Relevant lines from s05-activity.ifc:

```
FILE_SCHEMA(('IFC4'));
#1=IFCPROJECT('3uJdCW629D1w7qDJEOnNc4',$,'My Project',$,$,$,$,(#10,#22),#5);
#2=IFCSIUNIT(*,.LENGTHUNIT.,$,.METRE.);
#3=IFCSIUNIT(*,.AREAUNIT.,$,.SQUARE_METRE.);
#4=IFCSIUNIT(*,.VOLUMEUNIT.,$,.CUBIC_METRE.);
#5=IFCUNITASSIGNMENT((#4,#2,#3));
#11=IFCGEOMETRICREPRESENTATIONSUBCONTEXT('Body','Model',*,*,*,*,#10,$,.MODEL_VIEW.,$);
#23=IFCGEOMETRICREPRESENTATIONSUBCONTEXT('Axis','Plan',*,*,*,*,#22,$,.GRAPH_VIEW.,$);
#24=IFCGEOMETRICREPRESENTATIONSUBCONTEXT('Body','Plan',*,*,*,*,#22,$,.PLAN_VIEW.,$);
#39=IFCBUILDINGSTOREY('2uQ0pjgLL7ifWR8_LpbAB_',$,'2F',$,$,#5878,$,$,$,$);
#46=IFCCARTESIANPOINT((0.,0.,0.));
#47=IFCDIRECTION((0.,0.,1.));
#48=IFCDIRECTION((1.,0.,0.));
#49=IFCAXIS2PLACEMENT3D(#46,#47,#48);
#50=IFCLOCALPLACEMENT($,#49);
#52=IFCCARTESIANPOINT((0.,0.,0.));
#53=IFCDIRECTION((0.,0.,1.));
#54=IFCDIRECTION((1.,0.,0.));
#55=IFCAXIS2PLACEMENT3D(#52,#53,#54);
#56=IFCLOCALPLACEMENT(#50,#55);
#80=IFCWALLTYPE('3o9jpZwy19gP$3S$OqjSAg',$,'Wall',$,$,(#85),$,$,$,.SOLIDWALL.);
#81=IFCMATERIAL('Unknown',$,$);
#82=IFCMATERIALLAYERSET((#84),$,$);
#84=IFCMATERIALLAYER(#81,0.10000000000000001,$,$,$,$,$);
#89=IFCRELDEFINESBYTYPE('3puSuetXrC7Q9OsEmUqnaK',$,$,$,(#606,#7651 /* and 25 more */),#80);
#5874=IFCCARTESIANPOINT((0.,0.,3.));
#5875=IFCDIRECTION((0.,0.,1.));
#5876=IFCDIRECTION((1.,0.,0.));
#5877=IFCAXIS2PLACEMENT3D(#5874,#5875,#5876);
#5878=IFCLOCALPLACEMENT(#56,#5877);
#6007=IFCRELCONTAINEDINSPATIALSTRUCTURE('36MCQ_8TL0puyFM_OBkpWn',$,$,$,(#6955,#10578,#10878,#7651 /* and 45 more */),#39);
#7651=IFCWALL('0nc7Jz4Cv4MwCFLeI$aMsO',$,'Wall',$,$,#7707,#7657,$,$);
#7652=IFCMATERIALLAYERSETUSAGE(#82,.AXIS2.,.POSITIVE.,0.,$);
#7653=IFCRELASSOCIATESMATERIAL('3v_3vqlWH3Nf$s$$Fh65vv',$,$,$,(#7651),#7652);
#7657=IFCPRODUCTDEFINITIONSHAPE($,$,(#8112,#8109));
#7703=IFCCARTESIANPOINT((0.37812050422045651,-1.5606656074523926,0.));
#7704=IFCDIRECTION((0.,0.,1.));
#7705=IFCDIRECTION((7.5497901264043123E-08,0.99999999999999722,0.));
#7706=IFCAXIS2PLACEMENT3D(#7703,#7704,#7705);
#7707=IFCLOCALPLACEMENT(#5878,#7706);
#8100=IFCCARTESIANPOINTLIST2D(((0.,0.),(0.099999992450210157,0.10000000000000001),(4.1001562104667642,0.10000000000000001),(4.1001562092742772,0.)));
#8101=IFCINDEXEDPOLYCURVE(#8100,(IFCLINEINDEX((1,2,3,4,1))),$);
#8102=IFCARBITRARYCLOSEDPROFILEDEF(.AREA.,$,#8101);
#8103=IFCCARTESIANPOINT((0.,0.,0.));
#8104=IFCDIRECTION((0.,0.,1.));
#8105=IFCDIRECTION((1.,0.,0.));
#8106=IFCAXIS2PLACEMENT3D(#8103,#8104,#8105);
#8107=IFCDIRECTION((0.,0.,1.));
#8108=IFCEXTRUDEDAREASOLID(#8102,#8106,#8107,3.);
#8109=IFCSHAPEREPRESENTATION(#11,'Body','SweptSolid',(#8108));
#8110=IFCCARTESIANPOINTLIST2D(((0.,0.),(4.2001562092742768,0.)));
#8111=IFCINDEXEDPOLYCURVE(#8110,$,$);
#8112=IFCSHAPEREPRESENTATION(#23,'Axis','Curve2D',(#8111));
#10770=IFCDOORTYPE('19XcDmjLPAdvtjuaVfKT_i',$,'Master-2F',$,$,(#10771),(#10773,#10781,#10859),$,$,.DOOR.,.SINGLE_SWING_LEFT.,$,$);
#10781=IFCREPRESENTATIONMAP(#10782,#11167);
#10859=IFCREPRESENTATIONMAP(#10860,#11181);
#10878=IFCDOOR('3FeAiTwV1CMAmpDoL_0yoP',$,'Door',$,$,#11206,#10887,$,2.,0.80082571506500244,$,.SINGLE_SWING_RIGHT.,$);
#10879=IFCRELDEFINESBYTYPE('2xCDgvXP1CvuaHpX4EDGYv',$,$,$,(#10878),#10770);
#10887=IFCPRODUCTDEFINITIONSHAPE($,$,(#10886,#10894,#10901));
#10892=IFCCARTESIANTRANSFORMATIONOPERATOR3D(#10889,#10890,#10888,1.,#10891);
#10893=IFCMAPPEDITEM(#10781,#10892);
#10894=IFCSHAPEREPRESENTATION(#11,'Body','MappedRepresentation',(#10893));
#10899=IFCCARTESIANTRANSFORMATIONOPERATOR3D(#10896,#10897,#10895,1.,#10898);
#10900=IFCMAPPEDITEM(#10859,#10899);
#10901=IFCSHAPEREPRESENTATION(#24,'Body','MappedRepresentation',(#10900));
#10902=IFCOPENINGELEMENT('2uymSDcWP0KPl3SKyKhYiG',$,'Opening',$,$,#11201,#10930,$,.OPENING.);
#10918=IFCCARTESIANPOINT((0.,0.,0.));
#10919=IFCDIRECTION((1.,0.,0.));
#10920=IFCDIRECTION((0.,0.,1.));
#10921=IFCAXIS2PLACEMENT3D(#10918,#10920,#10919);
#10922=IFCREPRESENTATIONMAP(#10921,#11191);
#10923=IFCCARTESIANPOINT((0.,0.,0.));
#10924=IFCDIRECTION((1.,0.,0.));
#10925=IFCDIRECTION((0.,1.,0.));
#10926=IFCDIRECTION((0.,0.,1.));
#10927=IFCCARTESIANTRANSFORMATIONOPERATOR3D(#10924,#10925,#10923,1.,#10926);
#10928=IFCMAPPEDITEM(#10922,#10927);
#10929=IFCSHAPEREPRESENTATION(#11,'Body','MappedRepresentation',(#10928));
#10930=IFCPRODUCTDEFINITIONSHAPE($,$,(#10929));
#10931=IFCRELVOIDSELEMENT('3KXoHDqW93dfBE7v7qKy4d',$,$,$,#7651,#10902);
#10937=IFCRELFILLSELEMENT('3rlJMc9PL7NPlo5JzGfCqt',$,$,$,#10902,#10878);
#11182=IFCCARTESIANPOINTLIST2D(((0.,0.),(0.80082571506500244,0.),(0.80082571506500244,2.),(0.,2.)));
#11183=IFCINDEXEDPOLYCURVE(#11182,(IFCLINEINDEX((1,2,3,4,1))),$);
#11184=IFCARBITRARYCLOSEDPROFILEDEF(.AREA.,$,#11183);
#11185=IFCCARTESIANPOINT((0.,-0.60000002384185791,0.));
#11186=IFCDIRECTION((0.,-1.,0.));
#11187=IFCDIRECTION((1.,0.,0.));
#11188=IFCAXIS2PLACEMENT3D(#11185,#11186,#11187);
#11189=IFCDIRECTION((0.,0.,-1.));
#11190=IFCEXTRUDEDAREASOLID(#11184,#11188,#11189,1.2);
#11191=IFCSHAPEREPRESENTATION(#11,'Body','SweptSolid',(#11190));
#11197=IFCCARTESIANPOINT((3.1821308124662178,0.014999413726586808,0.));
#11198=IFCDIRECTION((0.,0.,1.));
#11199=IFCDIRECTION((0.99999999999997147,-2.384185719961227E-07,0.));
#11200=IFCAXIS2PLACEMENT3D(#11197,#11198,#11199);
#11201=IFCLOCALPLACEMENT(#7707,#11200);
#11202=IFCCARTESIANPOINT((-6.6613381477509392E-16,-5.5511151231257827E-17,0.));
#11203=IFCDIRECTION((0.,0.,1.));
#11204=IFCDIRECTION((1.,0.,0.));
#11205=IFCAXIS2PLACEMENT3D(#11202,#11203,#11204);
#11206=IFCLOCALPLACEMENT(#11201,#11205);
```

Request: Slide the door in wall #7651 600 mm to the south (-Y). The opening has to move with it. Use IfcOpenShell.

```python
import ifcopenshell
import ifcopenshell.api.geometry
import ifcopenshell.util.placement
import ifcopenshell.util.unit

model = ifcopenshell.open("s05-activity.ifc")
unit_scale = ifcopenshell.util.unit.calculate_unit_scale(model)

door = model.by_guid("3FeAiTwV1CMAmpDoL_0yoP")
opening = door.FillsVoids[0].RelatingOpeningElement
wall = opening.VoidsElements[0].RelatingBuildingElement

wall_matrix = ifcopenshell.util.placement.get_local_placement(wall.ObjectPlacement)
shift = wall_matrix[:3, 0] * -0.6 / unit_scale
before = ifcopenshell.util.placement.get_local_placement(door.ObjectPlacement)[:3, 3].copy()

# The door is placed relative to its opening, so it follows when the opening moves.
matrix = ifcopenshell.util.placement.get_local_placement(opening.ObjectPlacement)
matrix[:3, 3] += shift
ifcopenshell.api.geometry.edit_object_placement(
    model, product=opening, matrix=matrix, is_si=False, should_transform_children=True
)

after = ifcopenshell.util.placement.get_local_placement(door.ObjectPlacement)[:3, 3]
print("door moved by", (after - before).round(3) + 0.0)

model.write("s05-activity_updated.ifc")
```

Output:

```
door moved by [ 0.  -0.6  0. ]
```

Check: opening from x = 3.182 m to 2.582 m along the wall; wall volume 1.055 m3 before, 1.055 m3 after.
